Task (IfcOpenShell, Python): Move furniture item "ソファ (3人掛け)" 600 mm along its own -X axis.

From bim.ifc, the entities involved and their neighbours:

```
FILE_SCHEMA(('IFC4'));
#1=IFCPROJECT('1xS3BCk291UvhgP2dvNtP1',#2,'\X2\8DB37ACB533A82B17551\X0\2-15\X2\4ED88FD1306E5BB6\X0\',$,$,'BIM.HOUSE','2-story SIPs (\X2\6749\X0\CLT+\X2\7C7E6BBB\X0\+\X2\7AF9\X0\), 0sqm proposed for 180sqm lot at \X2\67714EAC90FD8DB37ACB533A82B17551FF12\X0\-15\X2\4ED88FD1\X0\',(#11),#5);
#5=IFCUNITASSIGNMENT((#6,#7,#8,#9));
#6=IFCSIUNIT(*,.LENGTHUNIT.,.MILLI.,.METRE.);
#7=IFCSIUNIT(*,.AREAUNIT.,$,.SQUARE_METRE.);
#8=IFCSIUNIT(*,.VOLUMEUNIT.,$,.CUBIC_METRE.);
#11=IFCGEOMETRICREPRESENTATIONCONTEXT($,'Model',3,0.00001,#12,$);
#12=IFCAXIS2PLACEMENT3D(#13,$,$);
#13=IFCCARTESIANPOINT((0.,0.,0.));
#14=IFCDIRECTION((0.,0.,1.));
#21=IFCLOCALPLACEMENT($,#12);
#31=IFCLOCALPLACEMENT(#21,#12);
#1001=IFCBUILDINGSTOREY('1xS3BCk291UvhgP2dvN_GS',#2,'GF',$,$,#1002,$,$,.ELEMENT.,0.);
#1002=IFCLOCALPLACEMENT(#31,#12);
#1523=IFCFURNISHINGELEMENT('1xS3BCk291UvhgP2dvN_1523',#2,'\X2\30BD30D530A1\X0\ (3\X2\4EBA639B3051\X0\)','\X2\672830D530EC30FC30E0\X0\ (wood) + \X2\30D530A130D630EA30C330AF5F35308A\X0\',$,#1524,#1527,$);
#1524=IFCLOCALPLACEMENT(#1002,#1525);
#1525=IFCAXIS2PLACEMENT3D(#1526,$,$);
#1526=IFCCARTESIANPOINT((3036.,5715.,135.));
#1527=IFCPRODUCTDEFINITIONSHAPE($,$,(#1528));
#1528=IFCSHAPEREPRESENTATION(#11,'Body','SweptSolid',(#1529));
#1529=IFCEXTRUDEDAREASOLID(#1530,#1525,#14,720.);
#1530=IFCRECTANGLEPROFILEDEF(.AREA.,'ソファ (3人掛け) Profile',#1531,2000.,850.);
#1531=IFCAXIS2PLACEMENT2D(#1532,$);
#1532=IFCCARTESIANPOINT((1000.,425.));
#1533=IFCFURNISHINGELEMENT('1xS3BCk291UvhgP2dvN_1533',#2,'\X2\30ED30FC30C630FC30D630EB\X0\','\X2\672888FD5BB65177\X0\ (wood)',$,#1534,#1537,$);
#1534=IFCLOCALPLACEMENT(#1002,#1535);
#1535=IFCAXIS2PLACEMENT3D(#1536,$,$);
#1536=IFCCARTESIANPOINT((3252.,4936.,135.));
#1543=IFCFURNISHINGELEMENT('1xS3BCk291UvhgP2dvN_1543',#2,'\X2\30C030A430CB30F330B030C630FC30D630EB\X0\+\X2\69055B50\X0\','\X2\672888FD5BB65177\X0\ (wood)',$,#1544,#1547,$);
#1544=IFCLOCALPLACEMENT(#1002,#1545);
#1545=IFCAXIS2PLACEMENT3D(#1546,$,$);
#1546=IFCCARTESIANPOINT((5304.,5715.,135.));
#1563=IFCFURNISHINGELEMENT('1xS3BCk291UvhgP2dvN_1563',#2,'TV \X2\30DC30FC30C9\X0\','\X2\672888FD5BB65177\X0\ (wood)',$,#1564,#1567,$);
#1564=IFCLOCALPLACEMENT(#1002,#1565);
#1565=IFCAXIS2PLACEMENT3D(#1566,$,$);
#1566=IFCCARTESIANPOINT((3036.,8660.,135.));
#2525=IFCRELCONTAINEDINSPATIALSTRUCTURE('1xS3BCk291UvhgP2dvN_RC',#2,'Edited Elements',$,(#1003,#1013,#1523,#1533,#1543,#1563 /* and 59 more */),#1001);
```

```python
import ifcopenshell
import ifcopenshell.api.geometry
import ifcopenshell.util.placement

model = ifcopenshell.open("bim.ifc")

item = model.by_guid("1xS3BCk291UvhgP2dvN_1523")
matrix = ifcopenshell.util.placement.get_local_placement(item.ObjectPlacement)
matrix[:3, 3] -= matrix[:3, 0] * 600.0
ifcopenshell.api.geometry.edit_object_placement(model, product=item, matrix=matrix, is_si=False)

print(ifcopenshell.util.placement.get_local_placement(item.ObjectPlacement).round(3) + 0.0)

model.write("bim_v2.ifc")
```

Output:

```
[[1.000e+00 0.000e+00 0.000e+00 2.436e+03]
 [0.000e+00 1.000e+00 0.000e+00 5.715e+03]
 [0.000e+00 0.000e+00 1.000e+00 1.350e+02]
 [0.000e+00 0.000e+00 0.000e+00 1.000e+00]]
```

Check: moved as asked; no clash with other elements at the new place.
